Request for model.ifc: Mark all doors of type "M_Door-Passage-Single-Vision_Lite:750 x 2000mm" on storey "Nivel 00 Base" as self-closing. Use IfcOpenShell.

First a look at what the model holds.

```python
import ifcopenshell
import ifcopenshell.util.element

model = ifcopenshell.open("model.ifc")
print(model.schema)
storey = next(s for s in model.by_type("IfcBuildingStorey") if s.Name == "Nivel 00 Base")
doors = [e for e in ifcopenshell.util.element.get_decomposition(storey) if e.is_a("IfcDoor")]
seen = {}
for e in doors:
    element_type = ifcopenshell.util.element.get_type(e)
    key = (element_type.Name if element_type != e and element_type else None, ifcopenshell.util.element.get_pset(e, "Pset_DoorCommon", "SelfClosing"))
    seen[key] = seen.get(key, 0) + 1
for (name, value), count in sorted(seen.items(), key=str):
    print(count, "x", name, "|", value)
```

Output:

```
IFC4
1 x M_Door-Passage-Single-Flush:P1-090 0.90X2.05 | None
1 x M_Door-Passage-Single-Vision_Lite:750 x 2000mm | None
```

```python
import ifcopenshell
import ifcopenshell.api.pset
import ifcopenshell.util.element

model = ifcopenshell.open("model.ifc")

storey = next(s for s in model.by_type("IfcBuildingStorey") if s.Name == "Nivel 00 Base")
doors = [e for e in ifcopenshell.util.element.get_decomposition(storey) if e.is_a("IfcDoor")]

count = 0
for e in doors:
    element_type = ifcopenshell.util.element.get_type(e)
    if element_type in (None, e) or element_type.Name != "M_Door-Passage-Single-Vision_Lite:750 x 2000mm":
        continue
    # add_pset returns the element's existing set when there is one.
    pset = ifcopenshell.api.pset.add_pset(model, product=e, name="Pset_DoorCommon")
    ifcopenshell.api.pset.edit_pset(model, pset=pset, properties={"SelfClosing": True})
    count += 1

print(count, "doors updated")

model.write("model_v2.ifc")
```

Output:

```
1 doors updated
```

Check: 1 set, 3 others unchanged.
